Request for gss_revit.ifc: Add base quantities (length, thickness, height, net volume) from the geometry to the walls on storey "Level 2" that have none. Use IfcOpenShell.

First a look at what the model holds.

```python
import ifcopenshell
import ifcopenshell.util.element
import ifcopenshell.util.unit

model = ifcopenshell.open("gss_revit.ifc")
print(model.schema)
for unit_type in ("LENGTHUNIT", "AREAUNIT", "VOLUMEUNIT"):
    print(unit_type, ifcopenshell.util.unit.calculate_unit_scale(model, unit_type))
storey = next(s for s in model.by_type("IfcBuildingStorey") if s.Name == "Level 2")
walls = [e for e in ifcopenshell.util.element.get_decomposition(storey) if e.is_a("IfcWall")]
for e in sorted(walls, key=lambda e: e.id()):
    print(e.id(), e.is_a(), e.Name, list(ifcopenshell.util.element.get_psets(e, qtos_only=True)), sep=" | ")
```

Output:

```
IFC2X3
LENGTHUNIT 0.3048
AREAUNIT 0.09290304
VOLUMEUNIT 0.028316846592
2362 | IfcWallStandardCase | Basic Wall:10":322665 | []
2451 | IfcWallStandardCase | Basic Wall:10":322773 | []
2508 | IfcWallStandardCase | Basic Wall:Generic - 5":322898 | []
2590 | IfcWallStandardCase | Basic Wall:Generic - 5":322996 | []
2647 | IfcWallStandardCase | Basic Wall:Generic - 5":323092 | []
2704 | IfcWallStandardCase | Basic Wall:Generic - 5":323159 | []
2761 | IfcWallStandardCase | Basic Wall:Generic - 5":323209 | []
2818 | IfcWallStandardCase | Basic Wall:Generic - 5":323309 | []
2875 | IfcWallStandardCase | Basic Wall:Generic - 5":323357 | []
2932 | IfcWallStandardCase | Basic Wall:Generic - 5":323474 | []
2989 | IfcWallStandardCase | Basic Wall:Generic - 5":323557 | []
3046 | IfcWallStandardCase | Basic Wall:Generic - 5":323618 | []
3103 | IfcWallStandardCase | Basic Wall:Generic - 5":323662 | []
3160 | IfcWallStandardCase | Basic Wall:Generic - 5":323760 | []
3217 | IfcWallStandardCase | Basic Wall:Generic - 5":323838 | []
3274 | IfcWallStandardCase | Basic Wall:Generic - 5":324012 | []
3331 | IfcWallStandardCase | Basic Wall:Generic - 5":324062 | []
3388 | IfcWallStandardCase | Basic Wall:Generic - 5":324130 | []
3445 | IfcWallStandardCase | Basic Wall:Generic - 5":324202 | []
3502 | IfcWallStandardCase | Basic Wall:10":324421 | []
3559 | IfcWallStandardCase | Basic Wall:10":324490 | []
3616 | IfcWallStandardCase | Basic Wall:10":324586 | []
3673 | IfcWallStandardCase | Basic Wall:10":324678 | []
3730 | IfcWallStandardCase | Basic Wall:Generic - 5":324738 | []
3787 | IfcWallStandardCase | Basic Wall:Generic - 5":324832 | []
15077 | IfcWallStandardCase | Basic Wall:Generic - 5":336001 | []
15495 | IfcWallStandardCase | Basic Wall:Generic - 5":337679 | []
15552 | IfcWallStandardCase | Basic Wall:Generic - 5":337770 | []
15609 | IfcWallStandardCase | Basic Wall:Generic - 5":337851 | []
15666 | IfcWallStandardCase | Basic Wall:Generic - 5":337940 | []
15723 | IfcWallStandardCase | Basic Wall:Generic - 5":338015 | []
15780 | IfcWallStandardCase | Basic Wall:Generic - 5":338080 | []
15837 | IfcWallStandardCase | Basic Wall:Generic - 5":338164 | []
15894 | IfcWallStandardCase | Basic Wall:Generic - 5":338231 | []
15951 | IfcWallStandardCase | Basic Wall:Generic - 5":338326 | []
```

```python
import ifcopenshell
import ifcopenshell.api.pset
import ifcopenshell.geom
import ifcopenshell.util.element
import ifcopenshell.util.shape
import ifcopenshell.util.unit

model = ifcopenshell.open("gss_revit.ifc")
unit_scale = ifcopenshell.util.unit.calculate_unit_scale(model)
volume_scale = ifcopenshell.util.unit.calculate_unit_scale(model, "VOLUMEUNIT")
settings = ifcopenshell.geom.settings()

storey = next(s for s in model.by_type("IfcBuildingStorey") if s.Name == "Level 2")
walls = [e for e in ifcopenshell.util.element.get_decomposition(storey) if e.is_a("IfcWall")]

for e in sorted(walls, key=lambda e: e.id()):
    if ifcopenshell.util.element.get_psets(e, qtos_only=True, should_inherit=False):
        continue
    # Geometry comes back in metres, in the element's own axes.
    shape = ifcopenshell.geom.create_shape(settings, e)
    values = {
        "Length": ifcopenshell.util.shape.get_x(shape.geometry) / unit_scale,
        "Width": ifcopenshell.util.shape.get_y(shape.geometry) / unit_scale,
        "Height": ifcopenshell.util.shape.get_z(shape.geometry) / unit_scale,
        "NetVolume": ifcopenshell.util.shape.get_volume(shape.geometry) / volume_scale,
    }
    qto = ifcopenshell.api.pset.add_qto(model, product=e, name="BaseQuantities")
    ifcopenshell.api.pset.edit_qto(model, qto=qto, properties=values)
    print(e.id(), {k: round(v, 3) for k, v in values.items()})

model.write("gss_revit_v2.ifc")
```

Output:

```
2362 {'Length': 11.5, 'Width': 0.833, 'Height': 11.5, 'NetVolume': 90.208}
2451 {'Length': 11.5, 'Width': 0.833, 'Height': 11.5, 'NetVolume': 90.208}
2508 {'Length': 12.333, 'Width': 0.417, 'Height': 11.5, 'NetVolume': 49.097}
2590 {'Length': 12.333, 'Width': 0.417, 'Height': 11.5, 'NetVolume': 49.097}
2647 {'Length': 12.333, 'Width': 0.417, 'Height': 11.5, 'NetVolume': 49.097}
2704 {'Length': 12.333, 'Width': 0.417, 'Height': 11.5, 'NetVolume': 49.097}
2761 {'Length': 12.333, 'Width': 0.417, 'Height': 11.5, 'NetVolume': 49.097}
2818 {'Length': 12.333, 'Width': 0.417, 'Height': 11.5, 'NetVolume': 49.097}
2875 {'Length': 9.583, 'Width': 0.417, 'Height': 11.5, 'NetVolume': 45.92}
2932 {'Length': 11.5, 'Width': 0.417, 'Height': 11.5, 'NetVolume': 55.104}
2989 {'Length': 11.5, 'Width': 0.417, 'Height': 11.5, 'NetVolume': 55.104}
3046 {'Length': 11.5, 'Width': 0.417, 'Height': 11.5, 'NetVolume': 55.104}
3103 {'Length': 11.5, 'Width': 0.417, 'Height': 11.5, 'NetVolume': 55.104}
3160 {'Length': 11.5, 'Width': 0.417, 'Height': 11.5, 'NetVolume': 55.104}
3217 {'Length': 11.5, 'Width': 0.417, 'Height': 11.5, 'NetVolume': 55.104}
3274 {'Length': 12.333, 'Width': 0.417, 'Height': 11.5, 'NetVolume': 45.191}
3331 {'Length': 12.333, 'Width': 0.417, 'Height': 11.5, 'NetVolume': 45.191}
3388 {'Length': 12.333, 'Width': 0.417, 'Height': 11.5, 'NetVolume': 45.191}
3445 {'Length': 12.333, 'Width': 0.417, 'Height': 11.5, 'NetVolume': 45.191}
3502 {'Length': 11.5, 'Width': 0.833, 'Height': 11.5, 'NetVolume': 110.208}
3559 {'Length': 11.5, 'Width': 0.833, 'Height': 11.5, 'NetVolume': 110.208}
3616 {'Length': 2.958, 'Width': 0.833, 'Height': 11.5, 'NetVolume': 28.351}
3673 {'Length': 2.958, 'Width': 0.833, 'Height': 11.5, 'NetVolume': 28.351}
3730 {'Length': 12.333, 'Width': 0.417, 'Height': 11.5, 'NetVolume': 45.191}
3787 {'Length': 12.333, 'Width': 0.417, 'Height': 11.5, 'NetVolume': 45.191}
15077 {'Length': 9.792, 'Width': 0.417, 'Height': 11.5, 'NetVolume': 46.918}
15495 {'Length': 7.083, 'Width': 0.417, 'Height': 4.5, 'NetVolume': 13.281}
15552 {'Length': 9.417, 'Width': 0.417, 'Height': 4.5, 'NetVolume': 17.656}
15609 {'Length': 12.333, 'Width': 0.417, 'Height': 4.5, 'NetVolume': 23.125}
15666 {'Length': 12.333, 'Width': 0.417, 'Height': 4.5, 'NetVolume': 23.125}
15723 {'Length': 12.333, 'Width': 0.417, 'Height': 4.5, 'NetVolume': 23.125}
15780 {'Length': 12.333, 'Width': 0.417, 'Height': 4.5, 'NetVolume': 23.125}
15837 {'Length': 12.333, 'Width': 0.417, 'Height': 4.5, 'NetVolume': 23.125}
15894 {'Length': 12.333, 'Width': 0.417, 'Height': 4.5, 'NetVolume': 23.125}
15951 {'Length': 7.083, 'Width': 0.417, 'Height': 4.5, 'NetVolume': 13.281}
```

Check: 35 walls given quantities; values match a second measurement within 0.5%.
